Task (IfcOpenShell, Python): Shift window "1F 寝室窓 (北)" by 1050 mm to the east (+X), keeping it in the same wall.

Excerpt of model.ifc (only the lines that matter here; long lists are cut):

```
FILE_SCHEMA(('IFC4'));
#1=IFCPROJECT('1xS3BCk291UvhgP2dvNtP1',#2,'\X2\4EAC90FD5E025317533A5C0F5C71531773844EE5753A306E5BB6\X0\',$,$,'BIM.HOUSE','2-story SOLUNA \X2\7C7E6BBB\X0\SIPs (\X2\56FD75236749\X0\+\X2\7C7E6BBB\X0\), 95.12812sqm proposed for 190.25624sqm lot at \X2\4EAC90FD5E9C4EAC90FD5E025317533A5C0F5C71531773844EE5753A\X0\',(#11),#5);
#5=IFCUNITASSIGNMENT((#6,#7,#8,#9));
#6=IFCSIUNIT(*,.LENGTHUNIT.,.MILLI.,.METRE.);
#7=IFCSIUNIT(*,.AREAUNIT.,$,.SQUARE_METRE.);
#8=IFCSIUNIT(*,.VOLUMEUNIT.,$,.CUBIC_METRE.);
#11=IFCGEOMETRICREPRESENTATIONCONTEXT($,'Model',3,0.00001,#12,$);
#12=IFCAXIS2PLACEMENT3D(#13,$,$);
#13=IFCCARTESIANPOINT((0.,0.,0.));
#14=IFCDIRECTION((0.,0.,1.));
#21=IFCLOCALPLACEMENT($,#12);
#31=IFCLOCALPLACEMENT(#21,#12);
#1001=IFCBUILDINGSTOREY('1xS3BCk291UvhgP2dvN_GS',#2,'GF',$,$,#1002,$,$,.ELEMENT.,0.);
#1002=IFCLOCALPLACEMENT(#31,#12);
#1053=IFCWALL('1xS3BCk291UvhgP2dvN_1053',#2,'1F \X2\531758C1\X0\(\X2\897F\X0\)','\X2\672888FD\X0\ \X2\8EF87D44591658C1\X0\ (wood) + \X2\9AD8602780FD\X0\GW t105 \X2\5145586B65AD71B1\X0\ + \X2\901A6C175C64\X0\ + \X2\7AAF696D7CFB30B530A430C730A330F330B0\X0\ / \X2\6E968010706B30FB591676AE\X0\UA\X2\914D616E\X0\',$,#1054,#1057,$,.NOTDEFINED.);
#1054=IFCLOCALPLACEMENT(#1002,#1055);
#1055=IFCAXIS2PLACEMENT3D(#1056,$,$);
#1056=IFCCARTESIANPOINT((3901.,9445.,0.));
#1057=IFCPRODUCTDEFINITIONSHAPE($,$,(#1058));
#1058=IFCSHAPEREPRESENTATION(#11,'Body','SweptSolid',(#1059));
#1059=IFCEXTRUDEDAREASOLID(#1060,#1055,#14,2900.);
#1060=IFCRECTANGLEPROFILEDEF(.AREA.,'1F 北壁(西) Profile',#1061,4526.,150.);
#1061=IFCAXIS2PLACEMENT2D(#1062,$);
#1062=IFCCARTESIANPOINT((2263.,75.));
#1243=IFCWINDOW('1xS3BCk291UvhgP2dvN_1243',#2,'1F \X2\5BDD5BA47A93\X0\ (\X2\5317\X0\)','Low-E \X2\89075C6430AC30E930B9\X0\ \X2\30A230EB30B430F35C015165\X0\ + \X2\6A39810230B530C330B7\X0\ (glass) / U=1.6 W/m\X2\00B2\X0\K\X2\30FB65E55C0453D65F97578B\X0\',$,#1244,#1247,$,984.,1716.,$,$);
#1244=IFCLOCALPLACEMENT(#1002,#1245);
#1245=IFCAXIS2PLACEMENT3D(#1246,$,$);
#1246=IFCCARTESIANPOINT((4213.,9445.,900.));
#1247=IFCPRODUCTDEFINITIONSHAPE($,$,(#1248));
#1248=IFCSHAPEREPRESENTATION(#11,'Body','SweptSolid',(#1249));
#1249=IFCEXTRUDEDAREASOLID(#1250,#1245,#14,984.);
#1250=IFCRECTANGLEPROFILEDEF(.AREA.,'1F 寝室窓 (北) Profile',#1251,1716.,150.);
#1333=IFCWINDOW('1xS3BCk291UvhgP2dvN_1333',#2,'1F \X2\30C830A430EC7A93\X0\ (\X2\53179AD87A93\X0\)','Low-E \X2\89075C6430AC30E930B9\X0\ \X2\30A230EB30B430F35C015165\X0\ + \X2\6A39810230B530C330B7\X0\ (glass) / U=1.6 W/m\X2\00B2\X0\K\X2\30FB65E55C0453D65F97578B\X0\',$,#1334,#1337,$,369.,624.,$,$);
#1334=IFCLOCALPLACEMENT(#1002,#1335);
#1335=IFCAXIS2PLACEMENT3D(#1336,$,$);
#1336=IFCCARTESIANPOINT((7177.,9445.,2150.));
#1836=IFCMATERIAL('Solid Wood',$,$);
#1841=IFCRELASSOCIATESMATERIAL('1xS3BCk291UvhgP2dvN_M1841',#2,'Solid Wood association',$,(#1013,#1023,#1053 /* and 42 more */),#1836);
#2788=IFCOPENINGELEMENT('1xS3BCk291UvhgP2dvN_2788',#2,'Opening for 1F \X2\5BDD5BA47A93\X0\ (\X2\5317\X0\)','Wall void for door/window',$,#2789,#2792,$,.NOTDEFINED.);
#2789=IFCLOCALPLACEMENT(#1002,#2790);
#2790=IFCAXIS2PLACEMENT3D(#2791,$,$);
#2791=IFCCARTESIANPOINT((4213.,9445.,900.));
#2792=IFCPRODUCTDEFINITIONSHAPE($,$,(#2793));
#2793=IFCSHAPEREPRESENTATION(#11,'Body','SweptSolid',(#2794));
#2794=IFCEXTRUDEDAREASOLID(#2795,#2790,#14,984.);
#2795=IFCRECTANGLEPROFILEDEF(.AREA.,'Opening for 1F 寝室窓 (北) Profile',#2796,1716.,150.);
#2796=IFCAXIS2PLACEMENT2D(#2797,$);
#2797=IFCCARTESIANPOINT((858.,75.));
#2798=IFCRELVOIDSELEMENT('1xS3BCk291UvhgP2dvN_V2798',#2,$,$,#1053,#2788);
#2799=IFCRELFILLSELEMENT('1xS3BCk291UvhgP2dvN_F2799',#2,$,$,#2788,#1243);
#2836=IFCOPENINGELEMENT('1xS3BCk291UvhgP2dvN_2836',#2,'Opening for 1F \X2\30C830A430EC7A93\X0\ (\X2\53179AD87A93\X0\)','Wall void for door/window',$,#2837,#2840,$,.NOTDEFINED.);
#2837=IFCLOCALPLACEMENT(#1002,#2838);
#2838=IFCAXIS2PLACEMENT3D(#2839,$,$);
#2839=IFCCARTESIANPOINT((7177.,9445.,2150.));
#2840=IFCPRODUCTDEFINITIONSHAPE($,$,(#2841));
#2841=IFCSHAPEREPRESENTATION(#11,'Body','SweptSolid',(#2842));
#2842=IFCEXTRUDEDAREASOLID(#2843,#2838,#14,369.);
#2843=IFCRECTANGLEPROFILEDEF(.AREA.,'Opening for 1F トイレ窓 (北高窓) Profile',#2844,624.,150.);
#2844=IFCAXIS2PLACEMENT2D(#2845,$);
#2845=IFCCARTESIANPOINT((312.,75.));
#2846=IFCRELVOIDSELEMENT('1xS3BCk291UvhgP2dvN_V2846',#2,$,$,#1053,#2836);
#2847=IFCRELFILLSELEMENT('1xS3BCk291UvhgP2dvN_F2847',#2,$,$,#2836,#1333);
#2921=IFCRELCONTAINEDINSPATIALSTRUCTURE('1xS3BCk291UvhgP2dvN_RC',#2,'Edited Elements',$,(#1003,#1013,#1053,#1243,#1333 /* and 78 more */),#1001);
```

```python
import ifcopenshell
import ifcopenshell.api.geometry
import ifcopenshell.util.placement

model = ifcopenshell.open("model.ifc")

window = model.by_guid("1xS3BCk291UvhgP2dvN_1243")
opening = window.FillsVoids[0].RelatingOpeningElement
wall = opening.VoidsElements[0].RelatingBuildingElement

wall_matrix = ifcopenshell.util.placement.get_local_placement(wall.ObjectPlacement)
shift = wall_matrix[:3, 0] * 1050.0
before = ifcopenshell.util.placement.get_local_placement(window.ObjectPlacement)[:3, 3].copy()

# The window is not placed relative to its opening, so move both.
for product in (opening, window):
    matrix = ifcopenshell.util.placement.get_local_placement(product.ObjectPlacement)
    matrix[:3, 3] += shift
    ifcopenshell.api.geometry.edit_object_placement(model, product=product, matrix=matrix, is_si=False)

after = ifcopenshell.util.placement.get_local_placement(window.ObjectPlacement)[:3, 3]
print("window moved by", (after - before).round(3) + 0.0)

model.write("model_edited.ifc")
```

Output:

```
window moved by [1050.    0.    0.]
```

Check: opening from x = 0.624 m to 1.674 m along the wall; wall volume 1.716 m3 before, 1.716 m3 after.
